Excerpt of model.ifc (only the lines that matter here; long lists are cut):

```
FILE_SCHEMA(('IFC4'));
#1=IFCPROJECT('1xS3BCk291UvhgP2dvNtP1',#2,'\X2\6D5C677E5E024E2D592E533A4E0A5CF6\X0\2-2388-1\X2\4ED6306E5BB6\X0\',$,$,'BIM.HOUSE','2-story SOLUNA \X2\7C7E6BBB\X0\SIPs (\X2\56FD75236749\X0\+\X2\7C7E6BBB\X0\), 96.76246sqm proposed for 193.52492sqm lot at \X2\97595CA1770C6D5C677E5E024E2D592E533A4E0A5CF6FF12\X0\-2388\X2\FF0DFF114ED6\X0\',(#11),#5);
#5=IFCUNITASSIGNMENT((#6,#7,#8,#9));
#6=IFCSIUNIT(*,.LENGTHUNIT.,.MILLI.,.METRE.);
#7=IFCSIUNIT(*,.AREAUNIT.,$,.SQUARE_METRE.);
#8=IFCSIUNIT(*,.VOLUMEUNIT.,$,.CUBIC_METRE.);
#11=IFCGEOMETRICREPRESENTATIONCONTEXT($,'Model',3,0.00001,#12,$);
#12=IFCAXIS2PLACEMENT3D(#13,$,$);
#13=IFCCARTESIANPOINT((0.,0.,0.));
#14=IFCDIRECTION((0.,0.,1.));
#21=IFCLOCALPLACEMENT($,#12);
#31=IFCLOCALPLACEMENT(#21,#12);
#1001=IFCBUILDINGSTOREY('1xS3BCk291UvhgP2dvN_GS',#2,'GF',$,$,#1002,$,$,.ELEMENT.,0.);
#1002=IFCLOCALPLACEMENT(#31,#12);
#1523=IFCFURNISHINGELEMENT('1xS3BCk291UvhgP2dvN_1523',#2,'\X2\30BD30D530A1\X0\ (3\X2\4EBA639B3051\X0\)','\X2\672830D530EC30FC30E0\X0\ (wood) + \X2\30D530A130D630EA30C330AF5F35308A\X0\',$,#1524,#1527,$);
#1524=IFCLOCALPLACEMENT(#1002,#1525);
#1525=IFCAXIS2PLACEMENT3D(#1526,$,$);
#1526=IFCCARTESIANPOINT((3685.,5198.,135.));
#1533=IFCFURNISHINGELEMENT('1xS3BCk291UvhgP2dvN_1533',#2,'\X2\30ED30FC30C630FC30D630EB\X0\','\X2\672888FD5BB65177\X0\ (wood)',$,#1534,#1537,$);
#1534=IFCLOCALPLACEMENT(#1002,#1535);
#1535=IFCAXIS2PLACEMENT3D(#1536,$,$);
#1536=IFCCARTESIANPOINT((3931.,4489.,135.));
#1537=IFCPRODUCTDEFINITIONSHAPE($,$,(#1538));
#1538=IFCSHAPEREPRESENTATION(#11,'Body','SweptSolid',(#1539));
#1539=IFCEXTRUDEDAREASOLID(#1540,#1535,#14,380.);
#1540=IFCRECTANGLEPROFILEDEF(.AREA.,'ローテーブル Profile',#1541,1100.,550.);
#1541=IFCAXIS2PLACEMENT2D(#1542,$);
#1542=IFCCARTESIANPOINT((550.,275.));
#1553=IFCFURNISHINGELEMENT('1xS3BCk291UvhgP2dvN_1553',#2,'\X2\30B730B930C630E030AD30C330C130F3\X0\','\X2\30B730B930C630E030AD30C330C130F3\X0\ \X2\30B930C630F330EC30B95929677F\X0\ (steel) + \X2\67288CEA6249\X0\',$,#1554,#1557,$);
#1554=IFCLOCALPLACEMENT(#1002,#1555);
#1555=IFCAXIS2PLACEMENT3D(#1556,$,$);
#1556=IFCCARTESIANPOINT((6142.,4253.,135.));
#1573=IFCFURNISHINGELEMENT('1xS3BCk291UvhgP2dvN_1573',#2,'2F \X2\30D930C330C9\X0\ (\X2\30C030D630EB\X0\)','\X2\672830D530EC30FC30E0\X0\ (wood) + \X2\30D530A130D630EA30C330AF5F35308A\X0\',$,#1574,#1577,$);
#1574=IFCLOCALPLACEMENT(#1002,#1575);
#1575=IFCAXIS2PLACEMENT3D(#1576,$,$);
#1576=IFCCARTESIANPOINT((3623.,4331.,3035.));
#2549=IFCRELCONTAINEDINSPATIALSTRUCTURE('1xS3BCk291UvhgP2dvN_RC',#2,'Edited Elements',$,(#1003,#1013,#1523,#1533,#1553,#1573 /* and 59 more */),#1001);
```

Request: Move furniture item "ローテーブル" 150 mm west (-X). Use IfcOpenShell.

```python
import ifcopenshell
import ifcopenshell.api.geometry
import ifcopenshell.util.placement
import ifcopenshell.util.unit

model = ifcopenshell.open("model.ifc")
unit_scale = ifcopenshell.util.unit.calculate_unit_scale(model)

item = model.by_id(1533)
matrix = ifcopenshell.util.placement.get_local_placement(item.ObjectPlacement)
matrix[0, 3] -= 0.15 / unit_scale
ifcopenshell.api.geometry.edit_object_placement(model, product=item, matrix=matrix, is_si=False)

print(ifcopenshell.util.placement.get_local_placement(item.ObjectPlacement).round(3) + 0.0)

model.write("model_rev.ifc")
```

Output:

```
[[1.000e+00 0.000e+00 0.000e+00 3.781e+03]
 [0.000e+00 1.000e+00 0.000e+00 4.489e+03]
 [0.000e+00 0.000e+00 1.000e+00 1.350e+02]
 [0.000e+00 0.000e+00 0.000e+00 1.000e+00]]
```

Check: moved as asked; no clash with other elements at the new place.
